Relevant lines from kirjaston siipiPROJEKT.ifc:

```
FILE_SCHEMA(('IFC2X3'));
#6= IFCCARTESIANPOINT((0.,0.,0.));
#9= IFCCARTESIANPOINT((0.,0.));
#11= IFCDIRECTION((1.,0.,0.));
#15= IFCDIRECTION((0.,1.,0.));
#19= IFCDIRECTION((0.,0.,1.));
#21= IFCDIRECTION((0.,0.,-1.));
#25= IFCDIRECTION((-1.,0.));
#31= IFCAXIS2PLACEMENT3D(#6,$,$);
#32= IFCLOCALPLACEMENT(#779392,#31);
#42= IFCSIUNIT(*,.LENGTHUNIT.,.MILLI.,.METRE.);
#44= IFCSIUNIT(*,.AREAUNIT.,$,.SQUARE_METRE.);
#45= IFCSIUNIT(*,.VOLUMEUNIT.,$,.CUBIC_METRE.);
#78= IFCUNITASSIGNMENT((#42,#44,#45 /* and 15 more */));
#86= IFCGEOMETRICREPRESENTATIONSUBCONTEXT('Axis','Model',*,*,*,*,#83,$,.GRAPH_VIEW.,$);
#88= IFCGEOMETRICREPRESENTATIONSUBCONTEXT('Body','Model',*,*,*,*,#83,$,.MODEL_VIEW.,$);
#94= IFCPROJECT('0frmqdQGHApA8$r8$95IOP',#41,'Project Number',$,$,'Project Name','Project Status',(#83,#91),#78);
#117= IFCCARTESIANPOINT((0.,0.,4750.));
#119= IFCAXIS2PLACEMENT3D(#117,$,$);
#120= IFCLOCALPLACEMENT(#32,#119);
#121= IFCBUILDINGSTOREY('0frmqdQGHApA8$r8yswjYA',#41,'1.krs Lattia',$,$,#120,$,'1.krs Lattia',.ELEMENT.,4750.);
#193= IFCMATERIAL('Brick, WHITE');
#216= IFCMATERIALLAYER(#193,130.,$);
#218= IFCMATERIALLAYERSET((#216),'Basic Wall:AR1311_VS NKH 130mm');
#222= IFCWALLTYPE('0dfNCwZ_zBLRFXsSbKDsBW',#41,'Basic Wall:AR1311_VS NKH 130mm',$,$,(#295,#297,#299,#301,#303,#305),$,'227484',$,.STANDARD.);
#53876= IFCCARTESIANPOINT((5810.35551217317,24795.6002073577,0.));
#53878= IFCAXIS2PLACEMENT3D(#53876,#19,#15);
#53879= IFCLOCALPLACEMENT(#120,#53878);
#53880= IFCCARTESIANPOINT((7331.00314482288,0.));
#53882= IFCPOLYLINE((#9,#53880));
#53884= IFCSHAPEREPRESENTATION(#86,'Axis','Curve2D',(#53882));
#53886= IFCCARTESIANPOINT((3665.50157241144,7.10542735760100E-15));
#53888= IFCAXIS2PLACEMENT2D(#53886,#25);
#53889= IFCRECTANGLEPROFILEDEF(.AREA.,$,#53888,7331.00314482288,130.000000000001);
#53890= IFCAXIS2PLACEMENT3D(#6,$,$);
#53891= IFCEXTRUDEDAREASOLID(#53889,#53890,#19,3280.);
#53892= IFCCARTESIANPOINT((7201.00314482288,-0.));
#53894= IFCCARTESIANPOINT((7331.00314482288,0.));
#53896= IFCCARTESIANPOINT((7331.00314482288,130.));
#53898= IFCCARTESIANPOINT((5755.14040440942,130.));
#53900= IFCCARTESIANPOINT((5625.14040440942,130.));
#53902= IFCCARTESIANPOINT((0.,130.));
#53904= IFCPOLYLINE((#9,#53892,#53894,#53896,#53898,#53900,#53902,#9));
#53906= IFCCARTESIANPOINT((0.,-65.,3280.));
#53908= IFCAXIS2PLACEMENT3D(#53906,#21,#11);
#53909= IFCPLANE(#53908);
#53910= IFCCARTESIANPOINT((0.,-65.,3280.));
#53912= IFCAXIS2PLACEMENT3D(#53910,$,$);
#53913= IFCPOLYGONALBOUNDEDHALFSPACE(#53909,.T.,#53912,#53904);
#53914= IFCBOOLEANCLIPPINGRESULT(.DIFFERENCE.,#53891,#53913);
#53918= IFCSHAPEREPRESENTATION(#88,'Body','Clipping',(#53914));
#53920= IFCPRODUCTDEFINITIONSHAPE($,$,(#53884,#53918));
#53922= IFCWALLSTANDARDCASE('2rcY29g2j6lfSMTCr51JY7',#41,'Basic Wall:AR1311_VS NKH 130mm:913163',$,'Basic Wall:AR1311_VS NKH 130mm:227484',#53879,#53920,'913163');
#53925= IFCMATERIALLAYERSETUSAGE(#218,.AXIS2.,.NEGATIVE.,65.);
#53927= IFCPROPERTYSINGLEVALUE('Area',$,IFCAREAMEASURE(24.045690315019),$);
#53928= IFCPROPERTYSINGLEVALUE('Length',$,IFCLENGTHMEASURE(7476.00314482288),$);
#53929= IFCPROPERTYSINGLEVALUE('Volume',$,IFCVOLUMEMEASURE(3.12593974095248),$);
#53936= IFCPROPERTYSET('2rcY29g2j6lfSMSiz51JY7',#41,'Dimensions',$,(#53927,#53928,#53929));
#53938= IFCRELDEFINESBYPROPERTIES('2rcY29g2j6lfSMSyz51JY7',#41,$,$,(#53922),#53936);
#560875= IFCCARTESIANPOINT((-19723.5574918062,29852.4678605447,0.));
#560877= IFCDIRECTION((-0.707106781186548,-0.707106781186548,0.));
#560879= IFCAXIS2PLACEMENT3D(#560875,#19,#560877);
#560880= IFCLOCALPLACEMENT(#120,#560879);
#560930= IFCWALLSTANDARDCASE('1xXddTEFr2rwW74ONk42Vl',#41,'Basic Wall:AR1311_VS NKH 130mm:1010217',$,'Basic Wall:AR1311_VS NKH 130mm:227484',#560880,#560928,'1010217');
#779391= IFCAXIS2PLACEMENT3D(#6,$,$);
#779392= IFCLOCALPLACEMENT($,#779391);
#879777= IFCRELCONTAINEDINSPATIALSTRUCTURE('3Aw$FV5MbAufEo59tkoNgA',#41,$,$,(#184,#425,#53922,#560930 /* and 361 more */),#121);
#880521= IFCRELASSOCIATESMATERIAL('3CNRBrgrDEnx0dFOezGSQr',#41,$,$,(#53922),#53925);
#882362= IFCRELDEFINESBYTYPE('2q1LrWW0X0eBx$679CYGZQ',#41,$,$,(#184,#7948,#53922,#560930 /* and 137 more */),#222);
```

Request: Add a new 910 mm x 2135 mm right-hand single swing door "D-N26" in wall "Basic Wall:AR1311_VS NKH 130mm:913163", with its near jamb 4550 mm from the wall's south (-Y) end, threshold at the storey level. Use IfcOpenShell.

```python
import numpy as np
import ifcopenshell
import ifcopenshell.api.feature
import ifcopenshell.api.geometry
import ifcopenshell.api.pset
import ifcopenshell.api.root
import ifcopenshell.api.spatial
import ifcopenshell.api.type
import ifcopenshell.geom
import ifcopenshell.util.element
import ifcopenshell.util.placement
import ifcopenshell.util.representation
import ifcopenshell.util.shape
import ifcopenshell.util.unit

model = ifcopenshell.open("kirjaston siipiPROJEKT.ifc")
unit_scale = ifcopenshell.util.unit.calculate_unit_scale(model)
area_scale = ifcopenshell.util.unit.calculate_unit_scale(model, "AREAUNIT")
volume_scale = ifcopenshell.util.unit.calculate_unit_scale(model, "VOLUMEUNIT")
settings = ifcopenshell.geom.settings()


def volume(element):
    """Net volume in cubic metres, openings subtracted."""
    shape = ifcopenshell.geom.create_shape(settings, element)
    return ifcopenshell.util.shape.get_volume(shape.geometry)


wall = model.by_guid("2rcY29g2j6lfSMTCr51JY7")
storey = ifcopenshell.util.element.get_container(wall, ifc_class="IfcBuildingStorey")
context = ifcopenshell.util.representation.get_context(model, "Model", "Body", "MODEL_VIEW")
before = volume(wall)

width, height, from_end, sill = 0.91, 2.135, 4.55, 0.0  # metres

# The wall runs along its own X axis, and the end named is its -X end.
wall_shape = ifcopenshell.geom.create_shape(settings, wall)
x, y, z = ifcopenshell.util.shape.get_vertices(wall_shape.geometry).T
start = x.min() + from_end
face, thickness = float(y.min()), float(y.max() - y.min())
wall_matrix = ifcopenshell.util.placement.get_local_placement(wall.ObjectPlacement)
level = ifcopenshell.util.placement.get_local_placement(storey.ObjectPlacement)[2, 3]


def in_wall(x, y):
    """Placement at x, y metres in the wall's axes, at sill height."""
    matrix = wall_matrix.copy()
    matrix[:, 3] = wall_matrix @ np.array([x / unit_scale, y / unit_scale, 0.0, 1.0])
    matrix[2, 3] = level + sill / unit_scale
    return matrix


# Opening: a box that overshoots both wall faces by 50 mm.
opening = ifcopenshell.api.root.create_entity(model, ifc_class="IfcOpeningElement")
box = ifcopenshell.api.geometry.add_wall_representation(
    model, context=context, length=width, height=height, thickness=thickness + 0.1
)
ifcopenshell.api.geometry.assign_representation(model, product=opening, representation=box)
ifcopenshell.api.geometry.edit_object_placement(model, product=opening, matrix=in_wall(start, face - 0.05), is_si=False)
ifcopenshell.api.feature.add_feature(model, feature=opening, element=wall)

door = ifcopenshell.api.root.create_entity(model, ifc_class="IfcDoor", name="D-N26")
door.OverallWidth, door.OverallHeight = width / unit_scale, height / unit_scale
body = ifcopenshell.api.geometry.add_door_representation(
    model,
    context=context,
    overall_width=door.OverallWidth,
    overall_height=door.OverallHeight,
    operation_type="SINGLE_SWING_RIGHT",
    lining_properties={"LiningDepth": thickness / unit_scale, "ThresholdDepth": thickness / unit_scale},
)
ifcopenshell.api.geometry.assign_representation(model, product=door, representation=body)
ifcopenshell.api.spatial.assign_container(model, products=[door], relating_structure=storey)
fills = ifcopenshell.api.feature.add_filling(model, opening=opening, element=door)
fills.OwnerHistory = door.OwnerHistory  # required in IFC2X3

# IFC2X3 keeps the operation on the door style.
style = ifcopenshell.api.root.create_entity(model, ifc_class="IfcDoorStyle", name="D-N26")
style.OperationType, style.ConstructionType = "SINGLE_SWING_RIGHT", "NOTDEFINED"
style.ParameterTakesPrecedence = style.Sizeable = False
ifcopenshell.api.type.assign_type(model, related_objects=[door], relating_type=style)

# The lining spans the wall, so the door starts at the wall face.
ifcopenshell.api.geometry.edit_object_placement(model, product=door, matrix=in_wall(start, face), is_si=False)

after = volume(wall)

# Update the wall's stored quantities.
pset = model.by_id(ifcopenshell.util.element.get_pset(wall, "Dimensions", should_inherit=False)["id"])
ifcopenshell.api.pset.edit_pset(model, pset=pset, properties={
    "Area": model.create_entity("IfcAreaMeasure", after / thickness / area_scale),
    "Volume": model.create_entity("IfcVolumeMeasure", after / volume_scale),
})

print(f"wall volume {before:.3f} -> {after:.3f} m3")

model.write("kirjaston siipiPROJEKT_edited.ifc")
```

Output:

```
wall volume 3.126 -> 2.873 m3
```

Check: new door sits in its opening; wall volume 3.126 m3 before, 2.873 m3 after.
